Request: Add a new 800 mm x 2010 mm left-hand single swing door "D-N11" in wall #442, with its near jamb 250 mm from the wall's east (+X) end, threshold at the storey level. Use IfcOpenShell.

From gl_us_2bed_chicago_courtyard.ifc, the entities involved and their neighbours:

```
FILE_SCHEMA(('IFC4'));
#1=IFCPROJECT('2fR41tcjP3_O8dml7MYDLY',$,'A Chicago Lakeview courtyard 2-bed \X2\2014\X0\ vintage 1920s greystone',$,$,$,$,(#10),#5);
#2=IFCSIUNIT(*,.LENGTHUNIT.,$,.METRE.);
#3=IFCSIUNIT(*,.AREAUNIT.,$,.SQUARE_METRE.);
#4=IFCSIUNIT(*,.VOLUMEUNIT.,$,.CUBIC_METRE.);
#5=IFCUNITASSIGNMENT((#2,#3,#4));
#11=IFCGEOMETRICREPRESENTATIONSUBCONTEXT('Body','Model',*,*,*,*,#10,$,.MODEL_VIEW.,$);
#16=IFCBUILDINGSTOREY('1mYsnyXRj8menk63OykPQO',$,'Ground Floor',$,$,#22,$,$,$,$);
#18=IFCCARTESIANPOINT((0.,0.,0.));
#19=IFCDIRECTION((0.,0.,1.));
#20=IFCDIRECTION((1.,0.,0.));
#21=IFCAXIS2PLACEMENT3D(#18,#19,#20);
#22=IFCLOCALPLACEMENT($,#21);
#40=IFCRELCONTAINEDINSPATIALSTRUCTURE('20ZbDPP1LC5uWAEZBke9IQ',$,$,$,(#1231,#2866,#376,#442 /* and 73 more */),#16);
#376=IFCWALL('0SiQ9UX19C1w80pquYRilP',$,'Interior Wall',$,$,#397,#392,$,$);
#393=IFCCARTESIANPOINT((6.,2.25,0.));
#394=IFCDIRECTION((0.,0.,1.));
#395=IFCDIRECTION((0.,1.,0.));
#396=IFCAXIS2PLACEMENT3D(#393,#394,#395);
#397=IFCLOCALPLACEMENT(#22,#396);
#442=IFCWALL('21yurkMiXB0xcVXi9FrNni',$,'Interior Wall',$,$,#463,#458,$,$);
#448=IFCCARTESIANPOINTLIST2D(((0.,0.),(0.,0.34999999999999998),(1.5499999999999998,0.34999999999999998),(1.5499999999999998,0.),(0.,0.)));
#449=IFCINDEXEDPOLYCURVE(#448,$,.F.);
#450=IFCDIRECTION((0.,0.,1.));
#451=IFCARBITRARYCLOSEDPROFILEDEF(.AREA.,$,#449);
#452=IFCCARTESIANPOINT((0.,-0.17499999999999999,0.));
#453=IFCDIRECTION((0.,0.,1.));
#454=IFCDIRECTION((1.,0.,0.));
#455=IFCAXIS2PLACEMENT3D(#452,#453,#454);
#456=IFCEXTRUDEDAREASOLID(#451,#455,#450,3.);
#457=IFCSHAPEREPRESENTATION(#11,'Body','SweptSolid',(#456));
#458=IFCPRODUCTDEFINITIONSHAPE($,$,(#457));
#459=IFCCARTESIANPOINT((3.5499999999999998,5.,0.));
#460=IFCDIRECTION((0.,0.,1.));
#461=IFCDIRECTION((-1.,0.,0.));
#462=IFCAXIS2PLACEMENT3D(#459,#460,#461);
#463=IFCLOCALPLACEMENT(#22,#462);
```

```python
import numpy as np
import ifcopenshell
import ifcopenshell.api.feature
import ifcopenshell.api.geometry
import ifcopenshell.api.root
import ifcopenshell.api.spatial
import ifcopenshell.geom
import ifcopenshell.util.element
import ifcopenshell.util.placement
import ifcopenshell.util.representation
import ifcopenshell.util.shape
import ifcopenshell.util.unit

model = ifcopenshell.open("gl_us_2bed_chicago_courtyard.ifc")
unit_scale = ifcopenshell.util.unit.calculate_unit_scale(model)
settings = ifcopenshell.geom.settings()


def volume(element):
    """Net volume in cubic metres, openings subtracted."""
    shape = ifcopenshell.geom.create_shape(settings, element)
    return ifcopenshell.util.shape.get_volume(shape.geometry)


wall = model.by_guid("21yurkMiXB0xcVXi9FrNni")
storey = ifcopenshell.util.element.get_container(wall, ifc_class="IfcBuildingStorey")
context = ifcopenshell.util.representation.get_context(model, "Model", "Body", "MODEL_VIEW")
before = volume(wall)

width, height, from_end, sill = 0.8, 2.01, 0.25, 0.0  # metres

# The wall runs along its own X axis, and the end named is its -X end.
wall_shape = ifcopenshell.geom.create_shape(settings, wall)
x, y, z = ifcopenshell.util.shape.get_vertices(wall_shape.geometry).T
start = x.min() + from_end
face, thickness = float(y.min()), float(y.max() - y.min())
wall_matrix = ifcopenshell.util.placement.get_local_placement(wall.ObjectPlacement)
level = ifcopenshell.util.placement.get_local_placement(storey.ObjectPlacement)[2, 3]


def in_wall(x, y):
    """Placement at x, y metres in the wall's axes, at sill height."""
    matrix = wall_matrix.copy()
    matrix[:, 3] = wall_matrix @ np.array([x / unit_scale, y / unit_scale, 0.0, 1.0])
    matrix[2, 3] = level + sill / unit_scale
    return matrix


# Opening: a box that overshoots both wall faces by 50 mm.
opening = ifcopenshell.api.root.create_entity(model, ifc_class="IfcOpeningElement", predefined_type="OPENING")
box = ifcopenshell.api.geometry.add_wall_representation(
    model, context=context, length=width, height=height, thickness=thickness + 0.1
)
ifcopenshell.api.geometry.assign_representation(model, product=opening, representation=box)
ifcopenshell.api.geometry.edit_object_placement(model, product=opening, matrix=in_wall(start, face - 0.05), is_si=False)
ifcopenshell.api.feature.add_feature(model, feature=opening, element=wall)

door = ifcopenshell.api.root.create_entity(model, ifc_class="IfcDoor", name="D-N11", predefined_type="DOOR")
door.OverallWidth, door.OverallHeight = width / unit_scale, height / unit_scale
door.OperationType = "SINGLE_SWING_LEFT"
body = ifcopenshell.api.geometry.add_door_representation(
    model,
    context=context,
    overall_width=door.OverallWidth,
    overall_height=door.OverallHeight,
    operation_type="SINGLE_SWING_LEFT",
    lining_properties={"LiningDepth": thickness / unit_scale, "ThresholdDepth": thickness / unit_scale},
)
ifcopenshell.api.geometry.assign_representation(model, product=door, representation=body)
ifcopenshell.api.spatial.assign_container(model, products=[door], relating_structure=storey)
ifcopenshell.api.feature.add_filling(model, opening=opening, element=door)

# The lining spans the wall, so the door starts at the wall face.
ifcopenshell.api.geometry.edit_object_placement(model, product=door, matrix=in_wall(start, face), is_si=False)

after = volume(wall)

print(f"wall volume {before:.3f} -> {after:.3f} m3")

model.write("gl_us_2bed_chicago_courtyard_rev.ifc")
```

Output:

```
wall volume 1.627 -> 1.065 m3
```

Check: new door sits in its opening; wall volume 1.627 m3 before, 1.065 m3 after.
